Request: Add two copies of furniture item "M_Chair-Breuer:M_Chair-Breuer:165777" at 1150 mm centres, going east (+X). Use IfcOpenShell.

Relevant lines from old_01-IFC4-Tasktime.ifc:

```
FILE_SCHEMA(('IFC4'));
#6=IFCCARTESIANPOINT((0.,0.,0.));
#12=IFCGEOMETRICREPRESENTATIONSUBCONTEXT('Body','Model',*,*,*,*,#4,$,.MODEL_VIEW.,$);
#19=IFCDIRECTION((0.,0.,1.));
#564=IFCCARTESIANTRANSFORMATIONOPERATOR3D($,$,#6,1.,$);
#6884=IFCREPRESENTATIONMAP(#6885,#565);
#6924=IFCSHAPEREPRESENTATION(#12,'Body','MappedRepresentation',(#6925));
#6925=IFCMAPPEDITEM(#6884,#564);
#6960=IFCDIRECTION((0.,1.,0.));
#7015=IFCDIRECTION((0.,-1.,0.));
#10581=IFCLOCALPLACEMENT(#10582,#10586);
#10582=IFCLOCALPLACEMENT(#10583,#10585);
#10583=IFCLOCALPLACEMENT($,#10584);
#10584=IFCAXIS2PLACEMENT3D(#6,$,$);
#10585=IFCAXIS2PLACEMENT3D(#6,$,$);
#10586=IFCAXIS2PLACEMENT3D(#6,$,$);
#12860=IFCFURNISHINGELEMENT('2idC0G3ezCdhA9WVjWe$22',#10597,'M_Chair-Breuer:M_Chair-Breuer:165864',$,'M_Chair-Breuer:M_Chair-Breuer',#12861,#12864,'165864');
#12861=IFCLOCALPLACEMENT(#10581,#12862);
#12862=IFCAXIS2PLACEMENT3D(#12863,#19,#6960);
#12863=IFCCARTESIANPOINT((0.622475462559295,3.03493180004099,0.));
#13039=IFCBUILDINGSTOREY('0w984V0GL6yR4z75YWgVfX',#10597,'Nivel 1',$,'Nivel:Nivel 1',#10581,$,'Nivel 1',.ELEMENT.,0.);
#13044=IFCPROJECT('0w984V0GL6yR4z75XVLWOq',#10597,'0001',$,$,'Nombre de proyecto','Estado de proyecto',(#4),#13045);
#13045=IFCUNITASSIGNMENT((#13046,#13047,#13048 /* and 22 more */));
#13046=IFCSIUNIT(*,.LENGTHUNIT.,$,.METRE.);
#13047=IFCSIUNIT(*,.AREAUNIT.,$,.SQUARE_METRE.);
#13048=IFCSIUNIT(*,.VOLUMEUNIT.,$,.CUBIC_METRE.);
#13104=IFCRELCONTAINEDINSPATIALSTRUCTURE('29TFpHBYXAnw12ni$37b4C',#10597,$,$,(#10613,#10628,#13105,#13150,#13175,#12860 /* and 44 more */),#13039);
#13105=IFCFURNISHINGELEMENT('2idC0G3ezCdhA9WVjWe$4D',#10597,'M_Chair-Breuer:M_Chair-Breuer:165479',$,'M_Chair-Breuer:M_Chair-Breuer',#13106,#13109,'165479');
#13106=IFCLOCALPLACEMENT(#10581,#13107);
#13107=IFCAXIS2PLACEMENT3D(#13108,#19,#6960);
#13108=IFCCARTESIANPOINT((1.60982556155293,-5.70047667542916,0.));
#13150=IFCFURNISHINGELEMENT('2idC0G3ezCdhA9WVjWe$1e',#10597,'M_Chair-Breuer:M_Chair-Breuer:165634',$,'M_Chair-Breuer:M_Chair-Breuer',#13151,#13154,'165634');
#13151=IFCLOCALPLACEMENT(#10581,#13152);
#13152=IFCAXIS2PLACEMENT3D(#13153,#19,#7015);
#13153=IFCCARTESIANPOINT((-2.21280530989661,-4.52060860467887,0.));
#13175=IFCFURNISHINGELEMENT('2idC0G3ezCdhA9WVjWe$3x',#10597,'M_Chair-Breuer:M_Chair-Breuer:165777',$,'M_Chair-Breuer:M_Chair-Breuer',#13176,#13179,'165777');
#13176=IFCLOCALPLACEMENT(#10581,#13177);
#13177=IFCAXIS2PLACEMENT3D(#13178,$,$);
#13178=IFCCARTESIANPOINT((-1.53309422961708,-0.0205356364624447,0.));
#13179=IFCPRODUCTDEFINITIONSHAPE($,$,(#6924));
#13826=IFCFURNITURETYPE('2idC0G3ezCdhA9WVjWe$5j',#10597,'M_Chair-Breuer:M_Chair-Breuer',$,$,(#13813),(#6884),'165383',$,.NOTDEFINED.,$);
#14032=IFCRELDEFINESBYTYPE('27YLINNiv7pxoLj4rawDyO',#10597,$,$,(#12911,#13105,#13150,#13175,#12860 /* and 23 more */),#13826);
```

```python
import numpy as np
import ifcopenshell
import ifcopenshell.api.geometry
import ifcopenshell.api.root
import ifcopenshell.util.element
import ifcopenshell.util.placement

model = ifcopenshell.open("old_01-IFC4-Tasktime.ifc")


def reuse_history(source, copy):
    """copy_class also copies each property set's owner history, people and application; keep the originals."""
    for rel in copy.IsDefinedBy:
        if rel.is_a("IfcRelDefinesByProperties") and (history := rel.RelatingPropertyDefinition.OwnerHistory):
            rel.RelatingPropertyDefinition.OwnerHistory = source.OwnerHistory
            ifcopenshell.util.element.remove_deep2(model, history)


source = model.by_guid("2idC0G3ezCdhA9WVjWe$3x")
base = ifcopenshell.util.placement.get_local_placement(source.ObjectPlacement)
step = np.array([1.0, 0.0, 0.0]) * 1.15

for i in range(1, 3):
    copy = ifcopenshell.api.root.copy_class(model, product=source)
    copy.Representation = ifcopenshell.util.element.copy_deep(
        model, source.Representation, exclude=["IfcGeometricRepresentationContext", "IfcRepresentationMap"]
    )
    copy.Name = "M_Chair-Breuer:M_Chair-Breuer"
    copy.Tag = None
    reuse_history(source, copy)
    matrix = base.copy()
    matrix[:3, 3] += i * step
    print("added at", matrix[:3, 3].round(3) + 0.0)
    ifcopenshell.api.geometry.edit_object_placement(model, product=copy, matrix=matrix, is_si=False)

model.write("old_01-IFC4-Tasktime_updated.ifc")
```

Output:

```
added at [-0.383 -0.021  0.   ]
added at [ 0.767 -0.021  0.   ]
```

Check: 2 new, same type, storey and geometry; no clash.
